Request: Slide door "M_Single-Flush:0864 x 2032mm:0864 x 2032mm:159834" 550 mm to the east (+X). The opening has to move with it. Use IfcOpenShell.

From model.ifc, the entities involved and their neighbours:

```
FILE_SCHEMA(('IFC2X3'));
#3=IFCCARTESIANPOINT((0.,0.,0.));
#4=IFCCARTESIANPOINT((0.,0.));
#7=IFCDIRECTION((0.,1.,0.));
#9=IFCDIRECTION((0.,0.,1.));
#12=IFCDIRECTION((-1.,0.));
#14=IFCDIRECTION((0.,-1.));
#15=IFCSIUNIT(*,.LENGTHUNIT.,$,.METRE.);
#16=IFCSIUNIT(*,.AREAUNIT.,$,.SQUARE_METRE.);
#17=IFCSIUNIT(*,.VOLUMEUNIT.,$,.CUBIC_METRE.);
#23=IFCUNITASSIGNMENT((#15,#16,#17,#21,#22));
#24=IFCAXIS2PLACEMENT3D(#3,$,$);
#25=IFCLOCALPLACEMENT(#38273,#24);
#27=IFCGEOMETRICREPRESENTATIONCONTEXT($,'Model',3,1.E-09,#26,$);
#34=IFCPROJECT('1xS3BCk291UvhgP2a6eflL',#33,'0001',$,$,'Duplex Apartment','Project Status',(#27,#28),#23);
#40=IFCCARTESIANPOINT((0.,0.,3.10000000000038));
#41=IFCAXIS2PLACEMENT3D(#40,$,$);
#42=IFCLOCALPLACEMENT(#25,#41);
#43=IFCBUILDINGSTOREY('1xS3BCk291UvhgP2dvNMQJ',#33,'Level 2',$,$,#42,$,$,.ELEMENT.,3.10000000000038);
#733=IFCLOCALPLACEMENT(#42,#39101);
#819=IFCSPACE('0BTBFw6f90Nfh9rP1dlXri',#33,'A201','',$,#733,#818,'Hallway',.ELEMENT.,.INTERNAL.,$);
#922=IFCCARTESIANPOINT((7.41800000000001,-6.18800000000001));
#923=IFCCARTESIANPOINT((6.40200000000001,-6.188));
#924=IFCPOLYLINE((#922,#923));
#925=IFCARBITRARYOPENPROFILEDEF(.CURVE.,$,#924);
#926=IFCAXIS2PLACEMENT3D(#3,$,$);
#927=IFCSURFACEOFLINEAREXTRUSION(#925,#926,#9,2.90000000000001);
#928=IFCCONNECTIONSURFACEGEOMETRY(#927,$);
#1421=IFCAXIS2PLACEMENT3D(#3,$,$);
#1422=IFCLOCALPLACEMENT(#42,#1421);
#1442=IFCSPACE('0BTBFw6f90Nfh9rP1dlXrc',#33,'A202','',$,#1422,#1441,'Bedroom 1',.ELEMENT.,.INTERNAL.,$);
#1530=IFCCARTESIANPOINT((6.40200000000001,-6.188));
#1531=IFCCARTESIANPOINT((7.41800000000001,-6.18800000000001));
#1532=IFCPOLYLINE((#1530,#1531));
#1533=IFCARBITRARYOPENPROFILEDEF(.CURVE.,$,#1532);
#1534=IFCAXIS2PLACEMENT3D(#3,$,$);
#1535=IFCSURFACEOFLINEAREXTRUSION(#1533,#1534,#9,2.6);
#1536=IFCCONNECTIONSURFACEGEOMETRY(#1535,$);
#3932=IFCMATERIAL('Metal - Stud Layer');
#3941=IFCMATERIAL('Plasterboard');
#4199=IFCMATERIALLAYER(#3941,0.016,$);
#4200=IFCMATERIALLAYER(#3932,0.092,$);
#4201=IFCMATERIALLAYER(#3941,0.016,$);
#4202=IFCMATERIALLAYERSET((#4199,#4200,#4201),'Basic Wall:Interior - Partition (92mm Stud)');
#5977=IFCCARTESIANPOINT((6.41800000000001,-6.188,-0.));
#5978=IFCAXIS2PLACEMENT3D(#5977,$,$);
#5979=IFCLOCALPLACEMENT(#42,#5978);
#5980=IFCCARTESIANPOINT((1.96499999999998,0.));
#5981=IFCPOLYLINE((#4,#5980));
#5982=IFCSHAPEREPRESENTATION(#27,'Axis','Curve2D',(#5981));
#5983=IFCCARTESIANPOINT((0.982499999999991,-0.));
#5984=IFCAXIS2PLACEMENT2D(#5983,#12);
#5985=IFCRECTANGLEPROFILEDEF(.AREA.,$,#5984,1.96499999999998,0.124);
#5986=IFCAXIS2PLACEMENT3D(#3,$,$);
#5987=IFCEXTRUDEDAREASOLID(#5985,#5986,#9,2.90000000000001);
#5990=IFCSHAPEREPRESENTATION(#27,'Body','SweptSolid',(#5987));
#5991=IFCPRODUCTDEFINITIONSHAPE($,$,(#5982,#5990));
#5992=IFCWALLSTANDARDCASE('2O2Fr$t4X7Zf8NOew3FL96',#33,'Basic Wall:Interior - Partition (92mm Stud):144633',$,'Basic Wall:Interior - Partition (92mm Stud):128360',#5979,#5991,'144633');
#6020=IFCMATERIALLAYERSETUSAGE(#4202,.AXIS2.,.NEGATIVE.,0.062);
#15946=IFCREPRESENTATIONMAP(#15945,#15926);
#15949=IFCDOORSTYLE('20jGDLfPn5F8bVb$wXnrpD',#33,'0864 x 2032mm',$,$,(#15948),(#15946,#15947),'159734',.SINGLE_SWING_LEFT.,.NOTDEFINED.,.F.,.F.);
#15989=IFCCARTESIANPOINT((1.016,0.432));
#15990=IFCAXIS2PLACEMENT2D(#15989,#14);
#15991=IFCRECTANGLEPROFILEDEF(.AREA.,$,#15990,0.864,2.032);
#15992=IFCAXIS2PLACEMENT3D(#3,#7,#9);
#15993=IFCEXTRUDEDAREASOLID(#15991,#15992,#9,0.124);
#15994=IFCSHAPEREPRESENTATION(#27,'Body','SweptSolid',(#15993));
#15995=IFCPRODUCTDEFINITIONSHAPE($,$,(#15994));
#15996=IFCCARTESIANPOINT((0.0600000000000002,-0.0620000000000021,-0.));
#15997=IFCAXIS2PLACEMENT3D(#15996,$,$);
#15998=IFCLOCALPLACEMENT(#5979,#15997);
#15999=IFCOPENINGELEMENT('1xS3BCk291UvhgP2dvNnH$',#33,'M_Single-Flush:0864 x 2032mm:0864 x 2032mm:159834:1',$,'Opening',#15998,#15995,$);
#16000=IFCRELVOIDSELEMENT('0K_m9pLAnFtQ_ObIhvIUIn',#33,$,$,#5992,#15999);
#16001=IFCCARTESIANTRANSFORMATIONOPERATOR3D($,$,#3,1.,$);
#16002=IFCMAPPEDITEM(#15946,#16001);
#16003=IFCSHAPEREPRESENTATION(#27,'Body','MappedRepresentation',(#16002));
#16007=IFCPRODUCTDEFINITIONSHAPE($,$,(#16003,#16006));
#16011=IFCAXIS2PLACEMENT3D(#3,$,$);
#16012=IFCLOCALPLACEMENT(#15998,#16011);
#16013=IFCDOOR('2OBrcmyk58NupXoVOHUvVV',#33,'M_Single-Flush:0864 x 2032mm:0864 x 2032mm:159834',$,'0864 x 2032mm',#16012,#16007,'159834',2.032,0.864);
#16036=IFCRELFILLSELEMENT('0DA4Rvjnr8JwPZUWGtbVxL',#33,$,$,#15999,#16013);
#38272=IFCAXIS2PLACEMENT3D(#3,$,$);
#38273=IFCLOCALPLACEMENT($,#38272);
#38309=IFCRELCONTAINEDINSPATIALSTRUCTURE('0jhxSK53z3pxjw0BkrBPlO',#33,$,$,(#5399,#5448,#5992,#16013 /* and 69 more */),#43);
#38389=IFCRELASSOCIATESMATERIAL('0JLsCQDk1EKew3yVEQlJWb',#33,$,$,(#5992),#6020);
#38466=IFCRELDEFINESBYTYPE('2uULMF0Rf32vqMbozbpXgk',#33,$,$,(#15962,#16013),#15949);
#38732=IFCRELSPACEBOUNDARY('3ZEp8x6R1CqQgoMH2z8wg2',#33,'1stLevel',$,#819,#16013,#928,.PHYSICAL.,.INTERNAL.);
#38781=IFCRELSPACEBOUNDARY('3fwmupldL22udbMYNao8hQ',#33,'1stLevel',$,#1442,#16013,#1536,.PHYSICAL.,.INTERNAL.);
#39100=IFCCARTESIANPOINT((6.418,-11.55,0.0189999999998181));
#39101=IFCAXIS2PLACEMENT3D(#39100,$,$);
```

```python
import numpy as np
import ifcopenshell
import ifcopenshell.api.geometry
import ifcopenshell.util.placement

model = ifcopenshell.open("model.ifc")

door = model.by_guid("2OBrcmyk58NupXoVOHUvVV")
opening = door.FillsVoids[0].RelatingOpeningElement
wall = opening.VoidsElements[0].RelatingBuildingElement

wall_matrix = ifcopenshell.util.placement.get_local_placement(wall.ObjectPlacement)
shift = wall_matrix[:3, 0] * 0.55
before = ifcopenshell.util.placement.get_local_placement(door.ObjectPlacement)[:3, 3].copy()

# The door is placed relative to its opening, so it follows when the opening moves.
matrix = ifcopenshell.util.placement.get_local_placement(opening.ObjectPlacement)
matrix[:3, 3] += shift
ifcopenshell.api.geometry.edit_object_placement(
    model, product=opening, matrix=matrix, is_si=False, should_transform_children=True
)

# Space boundary surfaces are stored in each space's coordinates; move them too.
for rel in door.ProvidesBoundaries:
    if not rel.ConnectionGeometry:
        continue
    surface = rel.ConnectionGeometry.SurfaceOnRelatingElement
    space_matrix = ifcopenshell.util.placement.get_local_placement(rel.RelatingSpace.ObjectPlacement)
    point = np.array(surface.Position.Location.Coordinates) + space_matrix[:3, :3].T @ shift
    surface.Position = model.createIfcAxis2Placement3D(
        model.createIfcCartesianPoint(point.tolist()), surface.Position.Axis, surface.Position.RefDirection
    )

after = ifcopenshell.util.placement.get_local_placement(door.ObjectPlacement)[:3, 3]
print("door moved by", (after - before).round(3) + 0.0)

model.write("model_edited.ifc")
```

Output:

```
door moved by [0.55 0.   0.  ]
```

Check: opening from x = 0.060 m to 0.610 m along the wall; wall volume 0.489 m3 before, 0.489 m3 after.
